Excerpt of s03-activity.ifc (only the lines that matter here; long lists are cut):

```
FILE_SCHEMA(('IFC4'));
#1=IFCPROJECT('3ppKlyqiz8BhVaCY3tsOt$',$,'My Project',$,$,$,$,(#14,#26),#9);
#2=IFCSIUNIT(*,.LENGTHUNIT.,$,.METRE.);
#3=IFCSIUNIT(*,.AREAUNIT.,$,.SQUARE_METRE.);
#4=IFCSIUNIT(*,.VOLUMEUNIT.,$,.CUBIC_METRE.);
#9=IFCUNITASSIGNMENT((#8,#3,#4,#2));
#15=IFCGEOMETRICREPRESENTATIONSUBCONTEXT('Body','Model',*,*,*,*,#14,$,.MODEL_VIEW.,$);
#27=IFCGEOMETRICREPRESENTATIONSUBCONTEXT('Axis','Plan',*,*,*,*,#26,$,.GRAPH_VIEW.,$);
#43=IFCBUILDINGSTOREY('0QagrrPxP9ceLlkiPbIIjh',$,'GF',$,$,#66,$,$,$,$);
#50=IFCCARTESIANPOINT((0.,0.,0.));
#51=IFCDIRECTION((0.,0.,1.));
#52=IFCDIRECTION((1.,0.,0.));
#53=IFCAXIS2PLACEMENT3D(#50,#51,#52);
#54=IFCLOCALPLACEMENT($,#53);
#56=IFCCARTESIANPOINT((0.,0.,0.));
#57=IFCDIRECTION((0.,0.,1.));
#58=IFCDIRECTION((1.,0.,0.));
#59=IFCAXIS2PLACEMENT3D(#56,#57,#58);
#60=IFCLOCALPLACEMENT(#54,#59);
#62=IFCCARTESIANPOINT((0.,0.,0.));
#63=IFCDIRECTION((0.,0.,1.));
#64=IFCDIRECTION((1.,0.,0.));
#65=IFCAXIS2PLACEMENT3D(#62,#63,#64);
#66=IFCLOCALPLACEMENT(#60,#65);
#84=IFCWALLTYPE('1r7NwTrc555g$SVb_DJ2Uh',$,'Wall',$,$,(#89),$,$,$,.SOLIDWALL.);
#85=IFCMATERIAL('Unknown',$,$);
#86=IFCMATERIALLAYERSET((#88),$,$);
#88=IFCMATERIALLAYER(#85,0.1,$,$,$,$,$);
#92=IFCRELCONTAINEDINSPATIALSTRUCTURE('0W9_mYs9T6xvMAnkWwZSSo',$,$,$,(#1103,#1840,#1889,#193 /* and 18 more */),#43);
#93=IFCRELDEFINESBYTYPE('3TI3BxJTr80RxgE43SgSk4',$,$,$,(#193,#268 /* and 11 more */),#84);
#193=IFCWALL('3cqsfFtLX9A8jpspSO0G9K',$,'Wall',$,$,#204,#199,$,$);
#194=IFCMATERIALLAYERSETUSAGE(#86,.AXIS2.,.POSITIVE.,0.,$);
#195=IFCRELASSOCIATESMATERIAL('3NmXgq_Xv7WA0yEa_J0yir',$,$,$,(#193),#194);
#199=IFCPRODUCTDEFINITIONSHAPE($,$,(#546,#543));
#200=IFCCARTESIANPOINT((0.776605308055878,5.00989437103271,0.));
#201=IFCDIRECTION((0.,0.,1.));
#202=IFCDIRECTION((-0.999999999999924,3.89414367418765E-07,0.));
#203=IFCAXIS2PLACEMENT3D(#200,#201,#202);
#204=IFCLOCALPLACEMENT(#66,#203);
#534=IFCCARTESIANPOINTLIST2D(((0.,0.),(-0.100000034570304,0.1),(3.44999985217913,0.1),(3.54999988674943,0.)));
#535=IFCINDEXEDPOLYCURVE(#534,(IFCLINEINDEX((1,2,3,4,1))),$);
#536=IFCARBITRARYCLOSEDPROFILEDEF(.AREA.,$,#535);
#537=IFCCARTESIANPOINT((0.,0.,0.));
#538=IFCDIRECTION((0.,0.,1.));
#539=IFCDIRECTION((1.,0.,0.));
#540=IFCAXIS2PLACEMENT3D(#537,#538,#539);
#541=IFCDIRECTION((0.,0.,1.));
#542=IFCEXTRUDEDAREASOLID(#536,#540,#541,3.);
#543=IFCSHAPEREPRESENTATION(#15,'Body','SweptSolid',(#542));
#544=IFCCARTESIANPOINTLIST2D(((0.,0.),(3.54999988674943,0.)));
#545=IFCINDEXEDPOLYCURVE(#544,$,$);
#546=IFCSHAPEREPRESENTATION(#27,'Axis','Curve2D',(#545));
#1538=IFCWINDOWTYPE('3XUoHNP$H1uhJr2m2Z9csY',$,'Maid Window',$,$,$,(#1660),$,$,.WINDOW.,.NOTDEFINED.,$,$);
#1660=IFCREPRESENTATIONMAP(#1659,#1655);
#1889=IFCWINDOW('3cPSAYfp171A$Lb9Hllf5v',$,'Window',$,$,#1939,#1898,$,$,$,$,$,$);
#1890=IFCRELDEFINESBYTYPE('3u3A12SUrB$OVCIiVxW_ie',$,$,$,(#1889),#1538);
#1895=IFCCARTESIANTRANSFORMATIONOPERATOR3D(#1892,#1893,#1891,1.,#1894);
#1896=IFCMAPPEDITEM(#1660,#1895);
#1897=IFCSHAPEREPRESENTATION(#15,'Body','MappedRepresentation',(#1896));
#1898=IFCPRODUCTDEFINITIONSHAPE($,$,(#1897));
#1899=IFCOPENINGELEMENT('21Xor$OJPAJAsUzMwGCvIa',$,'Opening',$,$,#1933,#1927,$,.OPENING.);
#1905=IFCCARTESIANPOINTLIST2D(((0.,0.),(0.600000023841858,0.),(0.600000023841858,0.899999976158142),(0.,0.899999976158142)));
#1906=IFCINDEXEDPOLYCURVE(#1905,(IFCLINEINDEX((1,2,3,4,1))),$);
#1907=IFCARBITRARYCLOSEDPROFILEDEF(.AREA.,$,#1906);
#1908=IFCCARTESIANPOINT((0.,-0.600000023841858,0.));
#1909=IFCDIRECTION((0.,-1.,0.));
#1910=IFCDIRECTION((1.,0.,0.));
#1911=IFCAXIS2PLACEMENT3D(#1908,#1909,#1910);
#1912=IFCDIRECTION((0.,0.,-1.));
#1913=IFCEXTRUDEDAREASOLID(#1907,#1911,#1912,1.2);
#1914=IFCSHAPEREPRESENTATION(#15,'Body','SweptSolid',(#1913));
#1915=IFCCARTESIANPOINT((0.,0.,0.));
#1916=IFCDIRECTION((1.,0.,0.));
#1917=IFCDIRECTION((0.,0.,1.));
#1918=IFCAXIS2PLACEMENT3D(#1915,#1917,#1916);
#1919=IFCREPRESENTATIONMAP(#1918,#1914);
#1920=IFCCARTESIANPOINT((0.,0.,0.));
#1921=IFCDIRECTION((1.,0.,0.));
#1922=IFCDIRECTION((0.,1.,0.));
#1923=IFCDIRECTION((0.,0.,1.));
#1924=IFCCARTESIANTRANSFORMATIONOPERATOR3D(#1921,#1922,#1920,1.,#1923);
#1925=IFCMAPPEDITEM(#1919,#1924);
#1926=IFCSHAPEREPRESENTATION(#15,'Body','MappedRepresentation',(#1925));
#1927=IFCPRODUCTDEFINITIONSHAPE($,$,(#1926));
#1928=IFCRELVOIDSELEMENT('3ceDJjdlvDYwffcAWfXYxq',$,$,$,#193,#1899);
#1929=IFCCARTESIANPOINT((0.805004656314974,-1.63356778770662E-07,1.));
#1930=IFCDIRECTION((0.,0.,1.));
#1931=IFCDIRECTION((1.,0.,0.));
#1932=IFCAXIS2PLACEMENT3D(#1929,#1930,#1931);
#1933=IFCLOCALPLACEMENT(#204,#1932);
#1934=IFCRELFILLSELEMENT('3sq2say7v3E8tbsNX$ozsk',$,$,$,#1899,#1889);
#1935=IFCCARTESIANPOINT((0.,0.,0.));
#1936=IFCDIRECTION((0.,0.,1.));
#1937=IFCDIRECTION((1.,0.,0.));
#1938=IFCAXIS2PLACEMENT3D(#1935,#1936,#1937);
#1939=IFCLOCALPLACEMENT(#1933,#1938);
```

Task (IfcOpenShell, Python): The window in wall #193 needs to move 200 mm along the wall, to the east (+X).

```python
import ifcopenshell
import ifcopenshell.api.geometry
import ifcopenshell.util.placement
import ifcopenshell.util.unit

model = ifcopenshell.open("s03-activity.ifc")
unit_scale = ifcopenshell.util.unit.calculate_unit_scale(model)

window = model.by_guid("3cPSAYfp171A$Lb9Hllf5v")
opening = window.FillsVoids[0].RelatingOpeningElement
wall = opening.VoidsElements[0].RelatingBuildingElement

wall_matrix = ifcopenshell.util.placement.get_local_placement(wall.ObjectPlacement)
shift = wall_matrix[:3, 0] * -0.2 / unit_scale
before = ifcopenshell.util.placement.get_local_placement(window.ObjectPlacement)[:3, 3].copy()

# The window is placed relative to its opening, so it follows when the opening moves.
matrix = ifcopenshell.util.placement.get_local_placement(opening.ObjectPlacement)
matrix[:3, 3] += shift
ifcopenshell.api.geometry.edit_object_placement(
    model, product=opening, matrix=matrix, is_si=False, should_transform_children=True
)

after = ifcopenshell.util.placement.get_local_placement(window.ObjectPlacement)[:3, 3]
print("window moved by", (after - before).round(3) + 0.0)

model.write("s03-activity-out.ifc")
```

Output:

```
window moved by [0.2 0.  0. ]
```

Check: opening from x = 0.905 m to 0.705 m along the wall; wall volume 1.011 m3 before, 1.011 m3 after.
